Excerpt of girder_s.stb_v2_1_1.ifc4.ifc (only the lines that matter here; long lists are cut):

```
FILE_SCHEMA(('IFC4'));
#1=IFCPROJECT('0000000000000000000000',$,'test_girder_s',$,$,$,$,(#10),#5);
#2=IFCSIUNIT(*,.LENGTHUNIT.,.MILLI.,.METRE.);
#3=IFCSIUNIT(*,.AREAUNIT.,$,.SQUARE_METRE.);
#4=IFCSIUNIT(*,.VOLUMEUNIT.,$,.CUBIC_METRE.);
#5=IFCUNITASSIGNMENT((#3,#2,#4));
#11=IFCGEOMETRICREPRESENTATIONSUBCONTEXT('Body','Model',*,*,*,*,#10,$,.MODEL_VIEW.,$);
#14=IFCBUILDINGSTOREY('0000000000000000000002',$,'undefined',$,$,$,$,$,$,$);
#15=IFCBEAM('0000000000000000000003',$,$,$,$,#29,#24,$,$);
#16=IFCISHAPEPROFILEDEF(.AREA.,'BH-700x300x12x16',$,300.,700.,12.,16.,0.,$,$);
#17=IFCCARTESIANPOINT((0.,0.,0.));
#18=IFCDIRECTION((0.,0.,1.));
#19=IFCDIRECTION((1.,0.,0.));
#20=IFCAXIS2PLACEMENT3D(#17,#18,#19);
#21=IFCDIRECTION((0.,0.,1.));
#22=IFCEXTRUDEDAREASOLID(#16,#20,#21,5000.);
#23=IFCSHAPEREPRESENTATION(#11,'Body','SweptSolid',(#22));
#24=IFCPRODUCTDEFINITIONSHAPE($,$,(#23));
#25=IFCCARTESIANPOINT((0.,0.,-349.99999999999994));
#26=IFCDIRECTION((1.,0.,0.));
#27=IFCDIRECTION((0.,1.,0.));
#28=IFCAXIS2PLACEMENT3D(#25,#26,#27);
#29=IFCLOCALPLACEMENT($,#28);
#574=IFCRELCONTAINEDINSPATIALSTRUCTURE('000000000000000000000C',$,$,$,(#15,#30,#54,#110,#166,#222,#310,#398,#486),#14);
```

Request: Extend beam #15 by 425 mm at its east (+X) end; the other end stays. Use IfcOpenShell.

```python
import ifcopenshell
import ifcopenshell.util.representation
import ifcopenshell.util.unit

model = ifcopenshell.open("girder_s.stb_v2_1_1.ifc4.ifc")
unit_scale = ifcopenshell.util.unit.calculate_unit_scale(model)

member = model.by_id(15)
change = 0.425 / unit_scale

# The extrusion runs towards the end named, so only its depth changes.
body = ifcopenshell.util.representation.get_representation(member, "Model", "Body")
solid = body.Items[0]
old_length = solid.Depth
solid.Depth += change

print(f"length {old_length:g} -> {solid.Depth:g}")

model.write("girder_s.stb_v2_1_1.ifc4-out.ifc")
```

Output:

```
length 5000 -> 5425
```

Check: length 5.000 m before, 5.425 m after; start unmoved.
